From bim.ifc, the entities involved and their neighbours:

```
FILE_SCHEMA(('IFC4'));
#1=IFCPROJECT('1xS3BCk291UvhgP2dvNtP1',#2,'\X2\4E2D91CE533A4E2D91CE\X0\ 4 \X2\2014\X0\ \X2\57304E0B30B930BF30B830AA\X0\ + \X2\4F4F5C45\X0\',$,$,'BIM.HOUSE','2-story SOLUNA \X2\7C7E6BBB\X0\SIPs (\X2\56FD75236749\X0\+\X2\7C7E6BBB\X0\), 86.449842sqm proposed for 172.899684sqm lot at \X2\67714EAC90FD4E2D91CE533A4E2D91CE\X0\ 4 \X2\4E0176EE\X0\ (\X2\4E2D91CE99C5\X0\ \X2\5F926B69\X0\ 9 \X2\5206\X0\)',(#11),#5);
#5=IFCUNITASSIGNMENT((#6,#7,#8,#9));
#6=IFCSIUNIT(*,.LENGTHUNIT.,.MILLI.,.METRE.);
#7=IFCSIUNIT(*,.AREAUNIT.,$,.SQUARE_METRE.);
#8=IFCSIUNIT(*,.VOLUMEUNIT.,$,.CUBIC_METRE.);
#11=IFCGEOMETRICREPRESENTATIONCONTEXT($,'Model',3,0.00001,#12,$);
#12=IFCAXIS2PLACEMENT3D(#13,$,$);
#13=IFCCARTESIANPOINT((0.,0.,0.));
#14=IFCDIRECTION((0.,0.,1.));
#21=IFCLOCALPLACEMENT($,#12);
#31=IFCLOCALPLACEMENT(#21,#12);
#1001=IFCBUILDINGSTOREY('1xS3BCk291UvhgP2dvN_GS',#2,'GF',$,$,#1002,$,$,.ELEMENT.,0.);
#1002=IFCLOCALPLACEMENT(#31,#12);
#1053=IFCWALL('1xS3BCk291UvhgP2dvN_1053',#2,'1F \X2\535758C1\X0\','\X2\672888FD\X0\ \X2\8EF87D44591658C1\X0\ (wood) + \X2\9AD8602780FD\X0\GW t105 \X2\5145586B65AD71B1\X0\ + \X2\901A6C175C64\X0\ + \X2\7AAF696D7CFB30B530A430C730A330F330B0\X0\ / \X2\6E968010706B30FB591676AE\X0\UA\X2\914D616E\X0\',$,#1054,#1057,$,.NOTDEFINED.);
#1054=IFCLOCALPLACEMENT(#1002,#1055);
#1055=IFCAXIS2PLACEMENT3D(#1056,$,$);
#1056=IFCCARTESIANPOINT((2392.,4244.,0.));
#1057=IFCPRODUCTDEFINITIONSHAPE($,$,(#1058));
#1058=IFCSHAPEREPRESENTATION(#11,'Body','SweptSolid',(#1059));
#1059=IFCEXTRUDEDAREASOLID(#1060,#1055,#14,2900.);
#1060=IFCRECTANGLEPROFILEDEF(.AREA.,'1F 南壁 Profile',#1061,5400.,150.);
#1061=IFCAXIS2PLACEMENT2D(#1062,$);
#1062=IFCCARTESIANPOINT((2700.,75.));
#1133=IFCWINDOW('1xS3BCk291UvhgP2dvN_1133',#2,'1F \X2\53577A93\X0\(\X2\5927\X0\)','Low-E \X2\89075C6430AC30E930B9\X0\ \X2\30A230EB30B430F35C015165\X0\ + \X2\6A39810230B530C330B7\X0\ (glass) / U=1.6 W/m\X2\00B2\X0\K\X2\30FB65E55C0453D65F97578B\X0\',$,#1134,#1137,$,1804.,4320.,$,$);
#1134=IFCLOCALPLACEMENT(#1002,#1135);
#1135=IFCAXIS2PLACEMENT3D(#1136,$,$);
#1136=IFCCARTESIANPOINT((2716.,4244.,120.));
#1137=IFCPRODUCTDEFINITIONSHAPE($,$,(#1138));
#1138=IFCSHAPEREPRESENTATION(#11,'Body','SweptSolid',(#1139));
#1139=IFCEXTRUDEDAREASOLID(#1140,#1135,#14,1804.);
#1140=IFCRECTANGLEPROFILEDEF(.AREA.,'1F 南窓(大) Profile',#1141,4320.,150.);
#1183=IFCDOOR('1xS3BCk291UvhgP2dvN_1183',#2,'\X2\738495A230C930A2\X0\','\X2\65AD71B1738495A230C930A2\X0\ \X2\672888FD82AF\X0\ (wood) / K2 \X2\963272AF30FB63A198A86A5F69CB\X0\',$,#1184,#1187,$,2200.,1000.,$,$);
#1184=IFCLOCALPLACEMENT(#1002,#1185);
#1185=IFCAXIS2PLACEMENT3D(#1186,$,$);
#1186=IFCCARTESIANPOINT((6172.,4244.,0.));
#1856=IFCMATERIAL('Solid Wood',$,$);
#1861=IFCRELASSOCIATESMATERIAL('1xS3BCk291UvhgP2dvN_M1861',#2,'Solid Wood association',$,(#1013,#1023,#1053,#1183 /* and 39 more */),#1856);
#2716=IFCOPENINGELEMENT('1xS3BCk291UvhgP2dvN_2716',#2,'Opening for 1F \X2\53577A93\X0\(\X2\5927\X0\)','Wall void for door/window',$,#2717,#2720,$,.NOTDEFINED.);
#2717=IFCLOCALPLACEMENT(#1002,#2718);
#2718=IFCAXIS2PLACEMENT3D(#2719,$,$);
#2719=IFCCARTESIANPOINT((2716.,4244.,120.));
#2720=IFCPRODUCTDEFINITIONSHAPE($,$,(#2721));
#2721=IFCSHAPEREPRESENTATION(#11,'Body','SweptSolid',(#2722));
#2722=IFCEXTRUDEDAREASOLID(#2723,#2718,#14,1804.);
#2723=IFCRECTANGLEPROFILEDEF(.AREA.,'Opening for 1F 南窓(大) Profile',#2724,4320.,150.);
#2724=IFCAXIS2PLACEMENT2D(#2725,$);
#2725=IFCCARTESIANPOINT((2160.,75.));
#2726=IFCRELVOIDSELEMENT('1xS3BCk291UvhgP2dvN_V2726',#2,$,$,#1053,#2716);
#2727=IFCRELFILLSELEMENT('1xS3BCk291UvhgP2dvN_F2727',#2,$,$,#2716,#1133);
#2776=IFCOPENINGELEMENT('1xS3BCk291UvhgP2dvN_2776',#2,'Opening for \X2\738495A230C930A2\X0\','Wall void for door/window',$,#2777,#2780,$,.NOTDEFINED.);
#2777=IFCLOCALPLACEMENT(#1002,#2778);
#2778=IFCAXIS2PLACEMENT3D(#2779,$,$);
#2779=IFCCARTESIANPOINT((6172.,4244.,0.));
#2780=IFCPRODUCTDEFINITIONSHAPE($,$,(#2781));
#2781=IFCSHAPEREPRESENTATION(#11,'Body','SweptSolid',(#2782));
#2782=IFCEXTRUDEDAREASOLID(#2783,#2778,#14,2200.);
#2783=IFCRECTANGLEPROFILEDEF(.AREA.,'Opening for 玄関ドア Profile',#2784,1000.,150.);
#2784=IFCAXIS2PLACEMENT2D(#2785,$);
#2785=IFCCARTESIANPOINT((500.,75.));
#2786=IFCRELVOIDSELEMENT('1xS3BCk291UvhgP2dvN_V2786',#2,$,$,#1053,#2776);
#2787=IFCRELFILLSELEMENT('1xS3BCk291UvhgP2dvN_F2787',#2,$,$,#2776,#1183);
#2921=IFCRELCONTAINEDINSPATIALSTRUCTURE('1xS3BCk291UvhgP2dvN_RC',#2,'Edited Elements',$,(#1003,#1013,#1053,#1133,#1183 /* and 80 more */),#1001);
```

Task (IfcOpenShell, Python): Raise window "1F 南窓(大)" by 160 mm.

```python
import numpy as np
import ifcopenshell
import ifcopenshell.api.geometry
import ifcopenshell.util.placement
import ifcopenshell.util.unit

model = ifcopenshell.open("bim.ifc")
unit_scale = ifcopenshell.util.unit.calculate_unit_scale(model)

window = model.by_id(1133)
opening = window.FillsVoids[0].RelatingOpeningElement
dz = 0.16 / unit_scale

shift = np.array([0.0, 0.0, dz])
# The window is not placed relative to its opening, so move both.
for product in (opening, window):
    matrix = ifcopenshell.util.placement.get_local_placement(product.ObjectPlacement)
    matrix[:3, 3] += shift
    ifcopenshell.api.geometry.edit_object_placement(model, product=product, matrix=matrix, is_si=False)

print(f"moved by {dz * unit_scale:+.3f} m")

model.write("bim-out.ifc")
```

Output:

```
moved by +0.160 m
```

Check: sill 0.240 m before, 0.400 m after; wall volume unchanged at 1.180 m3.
